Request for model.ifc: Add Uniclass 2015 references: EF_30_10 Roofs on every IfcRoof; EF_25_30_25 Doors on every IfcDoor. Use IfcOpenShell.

First a look at what the model holds.

```python
import ifcopenshell

model = ifcopenshell.open("model.ifc")
print(model.schema)
print("classifications:", [c.Name for c in model.by_type("IfcClassification")])
for ifc_class in ("IfcDoor", "IfcRoof", "IfcStair", "IfcWall", "IfcWindow"):
    print(ifc_class, len(model.by_type(ifc_class)))
```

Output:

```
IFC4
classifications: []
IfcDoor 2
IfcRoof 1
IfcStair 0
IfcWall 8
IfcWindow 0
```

```python
import ifcopenshell
import ifcopenshell.api.classification

model = ifcopenshell.open("model.ifc")

system = ifcopenshell.api.classification.add_classification(model, classification="Uniclass 2015")

codes = {
    "IfcRoof": ("EF_30_10", "Roofs"),
    "IfcDoor": ("EF_25_30_25", "Doors"),
}
for ifc_class, (code, name) in codes.items():
    products = model.by_type(ifc_class)
    ifcopenshell.api.classification.add_reference(
        model, products=products, classification=system, identification=code, name=name
    )
    print(code, len(products))

model.write("model_v2.ifc")
```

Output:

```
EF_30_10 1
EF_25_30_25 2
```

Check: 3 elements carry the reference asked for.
